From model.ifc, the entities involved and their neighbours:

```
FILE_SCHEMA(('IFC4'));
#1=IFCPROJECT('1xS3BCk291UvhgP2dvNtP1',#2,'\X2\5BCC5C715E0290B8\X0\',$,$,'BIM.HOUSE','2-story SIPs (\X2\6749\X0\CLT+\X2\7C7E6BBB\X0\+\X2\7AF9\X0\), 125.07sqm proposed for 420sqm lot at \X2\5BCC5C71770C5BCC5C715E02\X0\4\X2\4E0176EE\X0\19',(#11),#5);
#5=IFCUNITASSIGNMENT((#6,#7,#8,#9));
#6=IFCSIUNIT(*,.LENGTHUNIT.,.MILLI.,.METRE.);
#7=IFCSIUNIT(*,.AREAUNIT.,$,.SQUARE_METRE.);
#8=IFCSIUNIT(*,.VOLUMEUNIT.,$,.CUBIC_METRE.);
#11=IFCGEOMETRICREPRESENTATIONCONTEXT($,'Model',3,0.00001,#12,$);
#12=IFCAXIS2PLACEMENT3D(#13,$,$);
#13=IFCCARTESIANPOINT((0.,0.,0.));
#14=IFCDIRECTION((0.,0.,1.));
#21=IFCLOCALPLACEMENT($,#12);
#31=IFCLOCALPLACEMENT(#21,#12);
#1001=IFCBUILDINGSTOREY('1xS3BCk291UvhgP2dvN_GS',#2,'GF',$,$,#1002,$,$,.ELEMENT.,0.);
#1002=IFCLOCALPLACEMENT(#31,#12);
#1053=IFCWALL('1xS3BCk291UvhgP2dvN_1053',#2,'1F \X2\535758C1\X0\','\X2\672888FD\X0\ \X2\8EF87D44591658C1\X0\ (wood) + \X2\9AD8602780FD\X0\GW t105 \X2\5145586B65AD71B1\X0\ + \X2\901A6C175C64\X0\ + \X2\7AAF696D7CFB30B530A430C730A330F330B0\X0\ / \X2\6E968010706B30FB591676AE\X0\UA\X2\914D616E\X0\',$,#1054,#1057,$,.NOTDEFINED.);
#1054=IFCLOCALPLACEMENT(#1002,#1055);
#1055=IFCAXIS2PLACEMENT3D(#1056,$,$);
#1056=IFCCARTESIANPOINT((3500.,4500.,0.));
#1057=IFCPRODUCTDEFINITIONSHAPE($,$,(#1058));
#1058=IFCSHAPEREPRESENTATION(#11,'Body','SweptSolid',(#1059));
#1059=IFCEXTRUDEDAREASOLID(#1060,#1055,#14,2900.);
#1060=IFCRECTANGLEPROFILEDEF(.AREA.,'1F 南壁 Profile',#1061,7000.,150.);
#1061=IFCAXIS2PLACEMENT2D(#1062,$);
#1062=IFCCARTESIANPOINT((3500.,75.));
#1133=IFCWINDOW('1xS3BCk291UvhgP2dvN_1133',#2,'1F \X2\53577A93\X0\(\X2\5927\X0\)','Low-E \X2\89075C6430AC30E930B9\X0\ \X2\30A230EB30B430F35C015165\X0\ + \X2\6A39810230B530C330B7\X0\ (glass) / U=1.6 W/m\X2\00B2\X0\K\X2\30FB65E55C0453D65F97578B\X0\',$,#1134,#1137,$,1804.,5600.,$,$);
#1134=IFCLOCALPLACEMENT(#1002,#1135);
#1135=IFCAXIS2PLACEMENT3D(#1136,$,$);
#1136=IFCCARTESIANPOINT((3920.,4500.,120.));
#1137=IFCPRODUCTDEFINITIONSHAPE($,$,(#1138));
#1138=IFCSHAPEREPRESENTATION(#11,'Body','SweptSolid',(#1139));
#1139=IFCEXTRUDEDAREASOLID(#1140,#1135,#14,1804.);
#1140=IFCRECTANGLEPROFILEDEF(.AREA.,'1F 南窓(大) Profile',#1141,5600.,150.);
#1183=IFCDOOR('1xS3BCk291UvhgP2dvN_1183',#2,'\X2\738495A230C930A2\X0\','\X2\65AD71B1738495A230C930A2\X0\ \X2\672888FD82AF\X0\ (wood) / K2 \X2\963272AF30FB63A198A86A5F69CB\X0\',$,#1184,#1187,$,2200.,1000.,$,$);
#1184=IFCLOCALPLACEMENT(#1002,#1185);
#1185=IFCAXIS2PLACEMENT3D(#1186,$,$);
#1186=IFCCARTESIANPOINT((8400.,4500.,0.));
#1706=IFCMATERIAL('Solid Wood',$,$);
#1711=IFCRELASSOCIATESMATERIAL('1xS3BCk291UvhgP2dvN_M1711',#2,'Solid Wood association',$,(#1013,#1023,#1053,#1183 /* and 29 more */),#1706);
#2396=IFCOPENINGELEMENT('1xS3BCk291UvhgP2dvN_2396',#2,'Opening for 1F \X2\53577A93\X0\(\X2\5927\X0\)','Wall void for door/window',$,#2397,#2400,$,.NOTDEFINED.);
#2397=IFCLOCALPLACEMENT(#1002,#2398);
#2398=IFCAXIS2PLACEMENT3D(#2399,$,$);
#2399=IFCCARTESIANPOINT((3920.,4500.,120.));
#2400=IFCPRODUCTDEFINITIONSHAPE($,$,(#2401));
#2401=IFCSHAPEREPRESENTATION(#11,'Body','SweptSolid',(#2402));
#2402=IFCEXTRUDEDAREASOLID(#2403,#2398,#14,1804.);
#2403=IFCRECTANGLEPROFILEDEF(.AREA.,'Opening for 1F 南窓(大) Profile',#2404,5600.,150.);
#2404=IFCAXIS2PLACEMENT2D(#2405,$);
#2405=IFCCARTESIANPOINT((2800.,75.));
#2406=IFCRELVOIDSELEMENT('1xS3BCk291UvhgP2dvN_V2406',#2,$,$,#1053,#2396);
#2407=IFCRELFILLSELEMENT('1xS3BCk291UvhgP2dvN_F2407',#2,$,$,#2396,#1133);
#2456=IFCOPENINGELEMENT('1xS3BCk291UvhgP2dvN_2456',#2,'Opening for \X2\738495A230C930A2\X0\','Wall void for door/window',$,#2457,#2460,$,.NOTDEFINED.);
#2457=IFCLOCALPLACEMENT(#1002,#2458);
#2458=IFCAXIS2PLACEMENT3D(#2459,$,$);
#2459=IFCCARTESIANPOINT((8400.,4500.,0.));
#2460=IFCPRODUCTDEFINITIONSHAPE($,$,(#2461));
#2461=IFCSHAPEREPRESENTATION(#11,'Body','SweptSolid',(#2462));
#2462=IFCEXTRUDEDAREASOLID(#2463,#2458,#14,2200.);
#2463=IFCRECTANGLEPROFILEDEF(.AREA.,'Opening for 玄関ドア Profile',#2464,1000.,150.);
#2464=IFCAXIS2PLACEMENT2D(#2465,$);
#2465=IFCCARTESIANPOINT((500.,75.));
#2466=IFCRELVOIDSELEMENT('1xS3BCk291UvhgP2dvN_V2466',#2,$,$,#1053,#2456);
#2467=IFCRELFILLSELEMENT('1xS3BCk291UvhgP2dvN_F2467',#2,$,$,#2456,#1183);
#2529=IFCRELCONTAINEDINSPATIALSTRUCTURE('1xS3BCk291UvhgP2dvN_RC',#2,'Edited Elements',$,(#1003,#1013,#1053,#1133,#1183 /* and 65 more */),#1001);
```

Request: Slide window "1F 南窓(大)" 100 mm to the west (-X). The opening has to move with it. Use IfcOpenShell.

```python
import ifcopenshell
import ifcopenshell.api.geometry
import ifcopenshell.util.placement
import ifcopenshell.util.unit

model = ifcopenshell.open("model.ifc")
unit_scale = ifcopenshell.util.unit.calculate_unit_scale(model)

window = model.by_guid("1xS3BCk291UvhgP2dvN_1133")
opening = window.FillsVoids[0].RelatingOpeningElement
wall = opening.VoidsElements[0].RelatingBuildingElement

wall_matrix = ifcopenshell.util.placement.get_local_placement(wall.ObjectPlacement)
shift = wall_matrix[:3, 0] * -0.1 / unit_scale
before = ifcopenshell.util.placement.get_local_placement(window.ObjectPlacement)[:3, 3].copy()

# The window is not placed relative to its opening, so move both.
for product in (opening, window):
    matrix = ifcopenshell.util.placement.get_local_placement(product.ObjectPlacement)
    matrix[:3, 3] += shift
    ifcopenshell.api.geometry.edit_object_placement(model, product=product, matrix=matrix, is_si=False)

after = ifcopenshell.util.placement.get_local_placement(window.ObjectPlacement)[:3, 3]
print("window moved by", (after - before).round(3) + 0.0)

model.write("model_updated.ifc")
```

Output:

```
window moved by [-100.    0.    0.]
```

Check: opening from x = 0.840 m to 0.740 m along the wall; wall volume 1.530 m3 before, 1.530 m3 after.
